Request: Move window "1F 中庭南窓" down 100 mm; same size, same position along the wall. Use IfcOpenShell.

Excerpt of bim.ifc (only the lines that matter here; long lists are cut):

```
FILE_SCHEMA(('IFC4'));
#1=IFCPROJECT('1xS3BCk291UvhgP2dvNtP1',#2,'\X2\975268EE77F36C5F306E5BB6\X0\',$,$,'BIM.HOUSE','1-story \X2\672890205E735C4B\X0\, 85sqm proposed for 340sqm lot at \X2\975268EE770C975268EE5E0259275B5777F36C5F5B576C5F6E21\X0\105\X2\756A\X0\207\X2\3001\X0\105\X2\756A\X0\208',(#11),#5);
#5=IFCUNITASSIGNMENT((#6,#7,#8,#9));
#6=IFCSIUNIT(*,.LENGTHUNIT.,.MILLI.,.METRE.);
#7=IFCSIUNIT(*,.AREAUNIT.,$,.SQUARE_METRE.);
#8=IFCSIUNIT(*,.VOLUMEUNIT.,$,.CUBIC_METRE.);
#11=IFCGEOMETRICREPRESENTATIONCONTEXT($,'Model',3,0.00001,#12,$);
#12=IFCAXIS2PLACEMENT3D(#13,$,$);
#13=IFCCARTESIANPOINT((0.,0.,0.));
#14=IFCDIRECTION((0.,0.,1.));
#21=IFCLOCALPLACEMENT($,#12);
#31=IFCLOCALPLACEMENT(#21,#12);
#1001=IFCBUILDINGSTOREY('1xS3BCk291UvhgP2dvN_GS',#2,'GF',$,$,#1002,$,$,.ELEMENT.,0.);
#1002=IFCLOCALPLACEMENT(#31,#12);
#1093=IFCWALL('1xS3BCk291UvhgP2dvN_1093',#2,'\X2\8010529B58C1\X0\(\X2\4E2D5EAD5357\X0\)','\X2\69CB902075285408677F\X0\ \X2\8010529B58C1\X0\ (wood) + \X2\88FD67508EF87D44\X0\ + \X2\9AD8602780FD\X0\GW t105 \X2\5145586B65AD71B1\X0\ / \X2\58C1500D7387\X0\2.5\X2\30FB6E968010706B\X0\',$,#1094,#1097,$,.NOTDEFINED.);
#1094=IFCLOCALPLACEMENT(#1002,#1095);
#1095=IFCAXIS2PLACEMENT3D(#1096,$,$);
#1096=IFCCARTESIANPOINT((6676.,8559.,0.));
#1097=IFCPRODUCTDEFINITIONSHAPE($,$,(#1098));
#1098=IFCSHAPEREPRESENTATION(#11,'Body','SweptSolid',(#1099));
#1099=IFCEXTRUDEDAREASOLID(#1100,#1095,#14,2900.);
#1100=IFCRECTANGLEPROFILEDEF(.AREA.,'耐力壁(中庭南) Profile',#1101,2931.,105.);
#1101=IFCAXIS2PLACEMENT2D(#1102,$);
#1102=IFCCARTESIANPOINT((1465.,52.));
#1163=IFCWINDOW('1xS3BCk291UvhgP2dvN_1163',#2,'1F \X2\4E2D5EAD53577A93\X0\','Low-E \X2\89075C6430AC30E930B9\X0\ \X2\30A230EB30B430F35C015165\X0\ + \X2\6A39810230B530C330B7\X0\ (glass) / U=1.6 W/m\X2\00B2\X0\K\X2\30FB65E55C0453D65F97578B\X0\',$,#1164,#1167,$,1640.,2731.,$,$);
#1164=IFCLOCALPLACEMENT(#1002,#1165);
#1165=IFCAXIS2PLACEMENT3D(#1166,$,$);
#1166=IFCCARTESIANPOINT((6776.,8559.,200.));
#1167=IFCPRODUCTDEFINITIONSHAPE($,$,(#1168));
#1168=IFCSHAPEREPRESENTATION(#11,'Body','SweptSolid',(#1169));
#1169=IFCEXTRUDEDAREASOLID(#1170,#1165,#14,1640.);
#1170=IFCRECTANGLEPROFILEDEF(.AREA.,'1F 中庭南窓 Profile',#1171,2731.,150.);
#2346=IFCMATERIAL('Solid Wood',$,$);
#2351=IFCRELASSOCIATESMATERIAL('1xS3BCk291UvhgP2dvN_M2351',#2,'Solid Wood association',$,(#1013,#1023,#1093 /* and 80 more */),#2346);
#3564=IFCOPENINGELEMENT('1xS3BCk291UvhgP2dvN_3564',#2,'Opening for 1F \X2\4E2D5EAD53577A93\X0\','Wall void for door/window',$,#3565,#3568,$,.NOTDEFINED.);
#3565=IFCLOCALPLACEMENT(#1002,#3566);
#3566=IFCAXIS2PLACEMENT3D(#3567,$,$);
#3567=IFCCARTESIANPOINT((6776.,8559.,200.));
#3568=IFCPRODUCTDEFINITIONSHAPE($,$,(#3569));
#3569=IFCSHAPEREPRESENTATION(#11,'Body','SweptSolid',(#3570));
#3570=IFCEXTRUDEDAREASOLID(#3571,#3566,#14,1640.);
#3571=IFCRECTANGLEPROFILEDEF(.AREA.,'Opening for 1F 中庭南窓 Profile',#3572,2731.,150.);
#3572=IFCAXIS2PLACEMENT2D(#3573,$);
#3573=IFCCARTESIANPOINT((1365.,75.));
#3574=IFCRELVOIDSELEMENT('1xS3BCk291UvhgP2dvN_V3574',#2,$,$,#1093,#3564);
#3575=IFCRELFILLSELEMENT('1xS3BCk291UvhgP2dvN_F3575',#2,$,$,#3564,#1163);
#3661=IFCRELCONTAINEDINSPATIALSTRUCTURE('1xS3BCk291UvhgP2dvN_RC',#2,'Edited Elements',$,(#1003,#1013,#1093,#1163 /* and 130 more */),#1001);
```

```python
import numpy as np
import ifcopenshell
import ifcopenshell.api.geometry
import ifcopenshell.util.placement
import ifcopenshell.util.unit

model = ifcopenshell.open("bim.ifc")
unit_scale = ifcopenshell.util.unit.calculate_unit_scale(model)

window = model.by_id(1163)
opening = window.FillsVoids[0].RelatingOpeningElement
dz = -0.1 / unit_scale

shift = np.array([0.0, 0.0, dz])
# The window is not placed relative to its opening, so move both.
for product in (opening, window):
    matrix = ifcopenshell.util.placement.get_local_placement(product.ObjectPlacement)
    matrix[:3, 3] += shift
    ifcopenshell.api.geometry.edit_object_placement(model, product=product, matrix=matrix, is_si=False)

print(f"moved by {dz * unit_scale:+.3f} m")

model.write("bim_v2.ifc")
```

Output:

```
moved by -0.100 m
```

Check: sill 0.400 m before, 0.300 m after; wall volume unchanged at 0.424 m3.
